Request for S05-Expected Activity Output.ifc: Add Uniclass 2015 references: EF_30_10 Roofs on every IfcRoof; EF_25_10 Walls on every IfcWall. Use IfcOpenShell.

First a look at what the model holds.

```python
import ifcopenshell

model = ifcopenshell.open("S05-Expected Activity Output.ifc")
print(model.schema)
print("classifications:", [c.Name for c in model.by_type("IfcClassification")])
for ifc_class in ("IfcDoor", "IfcRoof", "IfcStair", "IfcWall", "IfcWindow"):
    print(ifc_class, len(model.by_type(ifc_class)))
```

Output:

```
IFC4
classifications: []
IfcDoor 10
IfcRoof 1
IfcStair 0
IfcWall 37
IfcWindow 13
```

```python
import ifcopenshell
import ifcopenshell.api.classification

model = ifcopenshell.open("S05-Expected Activity Output.ifc")

system = ifcopenshell.api.classification.add_classification(model, classification="Uniclass 2015")

codes = {
    "IfcRoof": ("EF_30_10", "Roofs"),
    "IfcWall": ("EF_25_10", "Walls"),
}
for ifc_class, (code, name) in codes.items():
    products = model.by_type(ifc_class)
    ifcopenshell.api.classification.add_reference(
        model, products=products, classification=system, identification=code, name=name
    )
    print(code, len(products))

model.write("S05-Expected Activity Output_updated.ifc")
```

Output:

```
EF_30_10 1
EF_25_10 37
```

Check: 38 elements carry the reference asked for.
